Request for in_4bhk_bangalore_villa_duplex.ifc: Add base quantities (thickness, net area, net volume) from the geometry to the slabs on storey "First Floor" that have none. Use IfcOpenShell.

First a look at what the model holds.

```python
import ifcopenshell
import ifcopenshell.util.element
import ifcopenshell.util.unit

model = ifcopenshell.open("in_4bhk_bangalore_villa_duplex.ifc")
print(model.schema)
for unit_type in ("LENGTHUNIT", "AREAUNIT", "VOLUMEUNIT"):
    print(unit_type, ifcopenshell.util.unit.calculate_unit_scale(model, unit_type))
storey = next(s for s in model.by_type("IfcBuildingStorey") if s.Name == "First Floor")
slabs = [e for e in ifcopenshell.util.element.get_decomposition(storey) if e.is_a("IfcSlab")]
for e in sorted(slabs, key=lambda e: e.id()):
    print(e.id(), e.is_a(), e.Name, list(ifcopenshell.util.element.get_psets(e, qtos_only=True)), sep=" | ")
```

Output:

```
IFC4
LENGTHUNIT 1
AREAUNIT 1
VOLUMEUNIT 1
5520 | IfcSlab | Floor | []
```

```python
import ifcopenshell
import ifcopenshell.api.pset
import ifcopenshell.geom
import ifcopenshell.util.element
import ifcopenshell.util.shape
import ifcopenshell.util.unit

model = ifcopenshell.open("in_4bhk_bangalore_villa_duplex.ifc")
unit_scale = ifcopenshell.util.unit.calculate_unit_scale(model)
area_scale = ifcopenshell.util.unit.calculate_unit_scale(model, "AREAUNIT")
volume_scale = ifcopenshell.util.unit.calculate_unit_scale(model, "VOLUMEUNIT")
settings = ifcopenshell.geom.settings()

storey = next(s for s in model.by_type("IfcBuildingStorey") if s.Name == "First Floor")
slabs = [e for e in ifcopenshell.util.element.get_decomposition(storey) if e.is_a("IfcSlab")]

for e in sorted(slabs, key=lambda e: e.id()):
    if ifcopenshell.util.element.get_psets(e, qtos_only=True, should_inherit=False):
        continue
    # Geometry comes back in metres, in the element's own axes.
    shape = ifcopenshell.geom.create_shape(settings, e)
    values = {
        "Width": ifcopenshell.util.shape.get_z(shape.geometry) / unit_scale,
        "NetArea": ifcopenshell.util.shape.get_footprint_area(shape.geometry) / area_scale,
        "NetVolume": ifcopenshell.util.shape.get_volume(shape.geometry) / volume_scale,
    }
    qto = ifcopenshell.api.pset.add_qto(model, product=e, name="Qto_SlabBaseQuantities")
    ifcopenshell.api.pset.edit_qto(model, qto=qto, properties=values)
    print(e.id(), {k: round(v, 3) for k, v in values.items()})

model.write("in_4bhk_bangalore_villa_duplex_rev.ifc")
```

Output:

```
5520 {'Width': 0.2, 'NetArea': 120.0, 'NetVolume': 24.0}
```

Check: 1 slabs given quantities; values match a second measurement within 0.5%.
